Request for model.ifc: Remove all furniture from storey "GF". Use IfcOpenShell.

First a look at what the model holds.

```python
import ifcopenshell
import ifcopenshell.util.element

model = ifcopenshell.open("model.ifc")
print(model.schema)
storey = next(s for s in model.by_type("IfcBuildingStorey") if s.Name == "GF")
furniture = [e for e in ifcopenshell.util.element.get_decomposition(storey) if e.is_a("IfcFurnishingElement")]
seen = {}
for e in furniture:
    element_type = ifcopenshell.util.element.get_type(e)
    name = element_type.Name if element_type not in (None, e) else None
    seen[name] = seen.get(name, 0) + 1
for name, count in sorted(seen.items(), key=str):
    print(count, "x", name)
```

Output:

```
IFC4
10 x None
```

```python
import ifcopenshell
import ifcopenshell.api.root
import ifcopenshell.util.element

model = ifcopenshell.open("model.ifc")

storey = next(s for s in model.by_type("IfcBuildingStorey") if s.Name == "GF")
furniture = [e for e in ifcopenshell.util.element.get_decomposition(storey) if e.is_a("IfcFurnishingElement")]

for e in furniture:
    ifcopenshell.api.root.remove_product(model, product=e)
print(len(furniture), "removed")

model.write("model_edited.ifc")
```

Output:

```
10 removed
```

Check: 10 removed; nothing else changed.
